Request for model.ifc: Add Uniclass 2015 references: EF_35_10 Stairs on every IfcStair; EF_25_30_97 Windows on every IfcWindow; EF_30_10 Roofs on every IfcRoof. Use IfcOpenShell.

First a look at what the model holds.

```python
import ifcopenshell

model = ifcopenshell.open("model.ifc")
print(model.schema)
print("classifications:", [c.Name for c in model.by_type("IfcClassification")])
for ifc_class in ("IfcDoor", "IfcRoof", "IfcStair", "IfcWall", "IfcWindow"):
    print(ifc_class, len(model.by_type(ifc_class)))
```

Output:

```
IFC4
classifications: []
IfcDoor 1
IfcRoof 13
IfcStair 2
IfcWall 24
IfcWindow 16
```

```python
import ifcopenshell
import ifcopenshell.api.classification

model = ifcopenshell.open("model.ifc")

system = ifcopenshell.api.classification.add_classification(model, classification="Uniclass 2015")

codes = {
    "IfcStair": ("EF_35_10", "Stairs"),
    "IfcWindow": ("EF_25_30_97", "Windows"),
    "IfcRoof": ("EF_30_10", "Roofs"),
}
for ifc_class, (code, name) in codes.items():
    products = model.by_type(ifc_class)
    ifcopenshell.api.classification.add_reference(
        model, products=products, classification=system, identification=code, name=name
    )
    print(code, len(products))

model.write("model-out.ifc")
```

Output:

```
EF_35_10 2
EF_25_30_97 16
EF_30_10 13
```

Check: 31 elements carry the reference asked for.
